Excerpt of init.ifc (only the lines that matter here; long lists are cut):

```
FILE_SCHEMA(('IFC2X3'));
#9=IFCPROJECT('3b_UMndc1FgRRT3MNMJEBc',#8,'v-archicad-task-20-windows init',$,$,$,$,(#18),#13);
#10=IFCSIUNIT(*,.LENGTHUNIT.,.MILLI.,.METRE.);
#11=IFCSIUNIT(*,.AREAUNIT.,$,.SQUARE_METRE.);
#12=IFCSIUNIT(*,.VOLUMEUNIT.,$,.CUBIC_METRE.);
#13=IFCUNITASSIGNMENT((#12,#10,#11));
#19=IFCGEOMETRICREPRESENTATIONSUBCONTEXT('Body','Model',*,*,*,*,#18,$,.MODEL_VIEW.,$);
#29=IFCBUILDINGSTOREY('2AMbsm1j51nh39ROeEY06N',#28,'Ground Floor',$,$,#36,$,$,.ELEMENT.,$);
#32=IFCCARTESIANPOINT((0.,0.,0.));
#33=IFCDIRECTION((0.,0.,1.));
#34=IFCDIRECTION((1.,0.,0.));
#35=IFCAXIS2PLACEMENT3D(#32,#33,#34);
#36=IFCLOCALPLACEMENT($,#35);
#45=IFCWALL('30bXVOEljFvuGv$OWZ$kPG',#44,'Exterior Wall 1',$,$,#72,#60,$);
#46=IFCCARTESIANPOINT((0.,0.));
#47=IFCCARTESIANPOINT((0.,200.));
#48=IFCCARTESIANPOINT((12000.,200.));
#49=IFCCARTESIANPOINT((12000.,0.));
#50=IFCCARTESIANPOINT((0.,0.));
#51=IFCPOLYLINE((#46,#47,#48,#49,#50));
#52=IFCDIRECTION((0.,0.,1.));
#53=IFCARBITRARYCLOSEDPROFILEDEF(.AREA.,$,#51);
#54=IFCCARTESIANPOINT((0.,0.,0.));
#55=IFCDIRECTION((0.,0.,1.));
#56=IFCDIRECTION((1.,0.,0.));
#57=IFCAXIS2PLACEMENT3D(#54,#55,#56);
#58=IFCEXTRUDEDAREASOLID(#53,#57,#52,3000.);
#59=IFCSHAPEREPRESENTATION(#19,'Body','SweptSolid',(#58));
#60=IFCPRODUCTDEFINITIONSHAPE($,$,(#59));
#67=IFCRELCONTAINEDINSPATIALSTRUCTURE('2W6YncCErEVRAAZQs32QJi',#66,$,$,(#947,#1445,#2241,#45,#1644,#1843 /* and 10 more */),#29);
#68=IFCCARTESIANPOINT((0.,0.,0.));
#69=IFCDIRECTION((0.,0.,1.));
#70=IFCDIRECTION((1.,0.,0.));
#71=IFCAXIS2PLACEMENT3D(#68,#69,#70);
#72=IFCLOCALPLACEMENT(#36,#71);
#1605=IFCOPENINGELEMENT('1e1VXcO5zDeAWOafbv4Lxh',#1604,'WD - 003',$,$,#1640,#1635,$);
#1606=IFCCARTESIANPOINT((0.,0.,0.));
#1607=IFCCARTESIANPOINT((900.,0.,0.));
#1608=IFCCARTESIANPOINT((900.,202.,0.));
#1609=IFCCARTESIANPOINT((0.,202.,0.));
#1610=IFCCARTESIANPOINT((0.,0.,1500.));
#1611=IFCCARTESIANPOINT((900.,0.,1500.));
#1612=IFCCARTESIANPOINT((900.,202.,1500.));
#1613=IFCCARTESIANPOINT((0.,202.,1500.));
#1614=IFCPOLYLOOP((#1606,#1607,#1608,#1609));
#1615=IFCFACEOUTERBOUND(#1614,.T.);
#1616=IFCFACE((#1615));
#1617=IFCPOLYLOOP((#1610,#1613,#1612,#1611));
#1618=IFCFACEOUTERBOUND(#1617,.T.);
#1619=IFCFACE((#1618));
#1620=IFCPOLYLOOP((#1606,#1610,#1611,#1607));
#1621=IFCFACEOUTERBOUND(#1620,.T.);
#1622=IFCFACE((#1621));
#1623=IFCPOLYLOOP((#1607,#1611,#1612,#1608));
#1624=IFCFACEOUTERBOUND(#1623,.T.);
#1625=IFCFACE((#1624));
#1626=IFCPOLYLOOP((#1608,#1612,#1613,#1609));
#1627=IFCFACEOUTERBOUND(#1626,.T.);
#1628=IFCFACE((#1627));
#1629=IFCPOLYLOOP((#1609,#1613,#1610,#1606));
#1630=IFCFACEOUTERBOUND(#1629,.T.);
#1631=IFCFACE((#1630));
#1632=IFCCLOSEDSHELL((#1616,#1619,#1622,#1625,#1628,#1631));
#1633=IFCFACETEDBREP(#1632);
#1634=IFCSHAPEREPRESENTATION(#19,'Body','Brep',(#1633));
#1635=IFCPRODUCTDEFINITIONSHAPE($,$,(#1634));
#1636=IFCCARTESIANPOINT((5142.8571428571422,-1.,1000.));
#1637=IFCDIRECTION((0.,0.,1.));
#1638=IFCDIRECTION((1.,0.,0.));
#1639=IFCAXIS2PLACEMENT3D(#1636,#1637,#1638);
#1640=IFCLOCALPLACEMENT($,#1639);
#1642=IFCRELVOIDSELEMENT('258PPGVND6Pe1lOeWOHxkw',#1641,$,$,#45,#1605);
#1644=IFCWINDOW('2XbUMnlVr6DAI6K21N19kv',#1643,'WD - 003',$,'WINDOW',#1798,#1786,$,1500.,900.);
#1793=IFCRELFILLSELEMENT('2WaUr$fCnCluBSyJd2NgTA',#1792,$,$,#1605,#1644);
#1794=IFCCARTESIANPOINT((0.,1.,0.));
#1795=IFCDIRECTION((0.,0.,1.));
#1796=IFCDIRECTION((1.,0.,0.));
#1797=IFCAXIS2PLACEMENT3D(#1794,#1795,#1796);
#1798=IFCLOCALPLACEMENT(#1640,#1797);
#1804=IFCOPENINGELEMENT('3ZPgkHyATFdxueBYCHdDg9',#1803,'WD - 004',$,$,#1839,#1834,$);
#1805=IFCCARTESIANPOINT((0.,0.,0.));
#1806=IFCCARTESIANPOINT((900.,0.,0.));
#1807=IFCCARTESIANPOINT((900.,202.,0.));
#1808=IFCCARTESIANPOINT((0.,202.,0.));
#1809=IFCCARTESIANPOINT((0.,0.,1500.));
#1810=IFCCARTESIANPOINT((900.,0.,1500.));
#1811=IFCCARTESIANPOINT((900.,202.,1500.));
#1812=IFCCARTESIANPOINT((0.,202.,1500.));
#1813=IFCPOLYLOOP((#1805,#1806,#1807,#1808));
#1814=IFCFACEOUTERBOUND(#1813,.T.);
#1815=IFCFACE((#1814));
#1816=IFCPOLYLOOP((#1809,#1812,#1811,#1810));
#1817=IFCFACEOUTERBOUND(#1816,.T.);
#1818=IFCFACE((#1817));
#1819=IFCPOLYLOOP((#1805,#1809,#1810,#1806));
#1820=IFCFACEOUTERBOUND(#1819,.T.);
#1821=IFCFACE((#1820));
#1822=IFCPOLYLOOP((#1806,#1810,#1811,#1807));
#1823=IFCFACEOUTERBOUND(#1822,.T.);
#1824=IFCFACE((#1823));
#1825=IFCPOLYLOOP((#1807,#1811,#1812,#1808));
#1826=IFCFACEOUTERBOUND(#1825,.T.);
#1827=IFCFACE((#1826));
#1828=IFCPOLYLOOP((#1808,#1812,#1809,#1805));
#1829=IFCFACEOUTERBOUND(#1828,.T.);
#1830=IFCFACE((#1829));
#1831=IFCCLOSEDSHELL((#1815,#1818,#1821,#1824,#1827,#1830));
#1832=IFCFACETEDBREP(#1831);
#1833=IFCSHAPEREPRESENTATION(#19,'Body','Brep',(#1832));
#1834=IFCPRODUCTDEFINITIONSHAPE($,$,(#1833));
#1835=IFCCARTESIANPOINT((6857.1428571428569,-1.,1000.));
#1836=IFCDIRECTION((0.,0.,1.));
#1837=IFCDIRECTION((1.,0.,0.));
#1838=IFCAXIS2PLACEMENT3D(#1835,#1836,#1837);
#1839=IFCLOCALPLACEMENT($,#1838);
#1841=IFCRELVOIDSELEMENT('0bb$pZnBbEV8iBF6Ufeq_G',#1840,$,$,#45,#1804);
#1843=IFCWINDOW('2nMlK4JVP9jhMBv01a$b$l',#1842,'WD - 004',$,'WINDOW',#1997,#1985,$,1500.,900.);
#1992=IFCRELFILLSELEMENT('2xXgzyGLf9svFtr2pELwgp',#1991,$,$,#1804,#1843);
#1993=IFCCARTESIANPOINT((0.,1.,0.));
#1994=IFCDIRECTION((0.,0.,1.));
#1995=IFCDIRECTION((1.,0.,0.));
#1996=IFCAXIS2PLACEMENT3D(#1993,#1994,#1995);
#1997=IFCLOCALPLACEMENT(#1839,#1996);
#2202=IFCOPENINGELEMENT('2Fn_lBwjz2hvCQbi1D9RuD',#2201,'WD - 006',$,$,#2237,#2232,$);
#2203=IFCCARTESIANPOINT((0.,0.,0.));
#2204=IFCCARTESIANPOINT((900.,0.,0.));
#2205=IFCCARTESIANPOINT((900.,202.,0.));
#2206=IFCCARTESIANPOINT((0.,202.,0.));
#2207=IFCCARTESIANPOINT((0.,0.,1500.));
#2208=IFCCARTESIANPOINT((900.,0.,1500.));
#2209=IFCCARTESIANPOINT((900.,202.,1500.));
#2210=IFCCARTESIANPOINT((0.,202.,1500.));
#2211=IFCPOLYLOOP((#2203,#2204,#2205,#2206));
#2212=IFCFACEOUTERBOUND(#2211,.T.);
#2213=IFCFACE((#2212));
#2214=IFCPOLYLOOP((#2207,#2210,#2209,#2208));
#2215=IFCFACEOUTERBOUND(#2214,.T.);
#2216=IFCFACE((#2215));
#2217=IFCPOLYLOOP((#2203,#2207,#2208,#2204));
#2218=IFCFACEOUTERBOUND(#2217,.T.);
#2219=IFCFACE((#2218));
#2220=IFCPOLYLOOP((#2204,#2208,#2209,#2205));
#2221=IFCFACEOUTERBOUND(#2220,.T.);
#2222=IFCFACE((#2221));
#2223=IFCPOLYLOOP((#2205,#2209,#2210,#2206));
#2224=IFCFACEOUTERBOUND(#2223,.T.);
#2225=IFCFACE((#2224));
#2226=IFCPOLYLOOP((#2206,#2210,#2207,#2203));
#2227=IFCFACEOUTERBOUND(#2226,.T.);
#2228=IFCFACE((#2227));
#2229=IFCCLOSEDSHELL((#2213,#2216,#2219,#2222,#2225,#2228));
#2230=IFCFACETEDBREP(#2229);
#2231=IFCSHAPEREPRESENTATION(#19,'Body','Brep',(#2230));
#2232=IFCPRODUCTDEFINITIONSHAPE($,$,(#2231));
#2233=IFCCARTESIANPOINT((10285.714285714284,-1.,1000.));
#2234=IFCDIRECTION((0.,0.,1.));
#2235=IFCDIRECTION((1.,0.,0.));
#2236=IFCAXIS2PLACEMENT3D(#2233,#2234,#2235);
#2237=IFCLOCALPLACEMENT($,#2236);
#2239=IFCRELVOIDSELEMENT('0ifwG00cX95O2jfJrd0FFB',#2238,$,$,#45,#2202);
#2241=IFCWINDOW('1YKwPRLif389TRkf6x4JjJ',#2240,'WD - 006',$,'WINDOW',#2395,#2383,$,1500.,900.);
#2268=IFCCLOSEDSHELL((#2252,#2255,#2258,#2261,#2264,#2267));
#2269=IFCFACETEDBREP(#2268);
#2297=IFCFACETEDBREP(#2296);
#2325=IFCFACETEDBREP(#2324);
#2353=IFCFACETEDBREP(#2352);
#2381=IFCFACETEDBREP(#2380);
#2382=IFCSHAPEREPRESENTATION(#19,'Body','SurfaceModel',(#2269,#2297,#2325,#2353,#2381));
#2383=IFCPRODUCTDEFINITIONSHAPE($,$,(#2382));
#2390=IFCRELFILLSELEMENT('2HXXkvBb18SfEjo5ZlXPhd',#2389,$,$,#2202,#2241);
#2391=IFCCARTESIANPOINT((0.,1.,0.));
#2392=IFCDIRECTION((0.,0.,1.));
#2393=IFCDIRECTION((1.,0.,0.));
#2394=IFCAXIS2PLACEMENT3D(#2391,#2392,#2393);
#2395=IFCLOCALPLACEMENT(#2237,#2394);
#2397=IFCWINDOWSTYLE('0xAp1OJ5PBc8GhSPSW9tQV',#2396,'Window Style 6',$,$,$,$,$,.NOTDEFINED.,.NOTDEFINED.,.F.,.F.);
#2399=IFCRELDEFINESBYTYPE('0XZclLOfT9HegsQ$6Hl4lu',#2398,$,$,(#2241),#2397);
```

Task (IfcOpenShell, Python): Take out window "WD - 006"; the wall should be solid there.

```python
import ifcopenshell
import ifcopenshell.api.feature
import ifcopenshell.api.root
import ifcopenshell.geom
import ifcopenshell.util.shape

model = ifcopenshell.open("init.ifc")
settings = ifcopenshell.geom.settings()


def volume(element):
    """Net volume in cubic metres, openings subtracted."""
    shape = ifcopenshell.geom.create_shape(settings, element)
    return ifcopenshell.util.shape.get_volume(shape.geometry)


window = model.by_guid("1YKwPRLif389TRkf6x4JjJ")
opening = window.FillsVoids[0].RelatingOpeningElement
wall = opening.VoidsElements[0].RelatingBuildingElement
before = volume(wall)

ifcopenshell.api.root.remove_product(model, product=window)
ifcopenshell.api.feature.remove_feature(model, feature=opening)

after = volume(wall)

print(f"wall volume {before:.3f} -> {after:.3f} m3")

model.write("init_rev.ifc")
```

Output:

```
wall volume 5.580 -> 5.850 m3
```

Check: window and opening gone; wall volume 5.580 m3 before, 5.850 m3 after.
